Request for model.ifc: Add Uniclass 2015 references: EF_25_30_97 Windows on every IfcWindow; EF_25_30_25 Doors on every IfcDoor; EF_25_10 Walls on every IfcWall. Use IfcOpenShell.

First a look at what the model holds.

```python
import ifcopenshell

model = ifcopenshell.open("model.ifc")
print(model.schema)
print("classifications:", [c.Name for c in model.by_type("IfcClassification")])
for ifc_class in ("IfcDoor", "IfcRoof", "IfcStair", "IfcWall", "IfcWindow"):
    print(ifc_class, len(model.by_type(ifc_class)))
```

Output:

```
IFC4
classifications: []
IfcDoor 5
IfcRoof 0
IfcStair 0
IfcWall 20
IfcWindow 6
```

```python
import ifcopenshell
import ifcopenshell.api.classification

model = ifcopenshell.open("model.ifc")

system = ifcopenshell.api.classification.add_classification(model, classification="Uniclass 2015")

codes = {
    "IfcWindow": ("EF_25_30_97", "Windows"),
    "IfcDoor": ("EF_25_30_25", "Doors"),
    "IfcWall": ("EF_25_10", "Walls"),
}
for ifc_class, (code, name) in codes.items():
    products = model.by_type(ifc_class)
    ifcopenshell.api.classification.add_reference(
        model, products=products, classification=system, identification=code, name=name
    )
    print(code, len(products))

model.write("model_edited.ifc")
```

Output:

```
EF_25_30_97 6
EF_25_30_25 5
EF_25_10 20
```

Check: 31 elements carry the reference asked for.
